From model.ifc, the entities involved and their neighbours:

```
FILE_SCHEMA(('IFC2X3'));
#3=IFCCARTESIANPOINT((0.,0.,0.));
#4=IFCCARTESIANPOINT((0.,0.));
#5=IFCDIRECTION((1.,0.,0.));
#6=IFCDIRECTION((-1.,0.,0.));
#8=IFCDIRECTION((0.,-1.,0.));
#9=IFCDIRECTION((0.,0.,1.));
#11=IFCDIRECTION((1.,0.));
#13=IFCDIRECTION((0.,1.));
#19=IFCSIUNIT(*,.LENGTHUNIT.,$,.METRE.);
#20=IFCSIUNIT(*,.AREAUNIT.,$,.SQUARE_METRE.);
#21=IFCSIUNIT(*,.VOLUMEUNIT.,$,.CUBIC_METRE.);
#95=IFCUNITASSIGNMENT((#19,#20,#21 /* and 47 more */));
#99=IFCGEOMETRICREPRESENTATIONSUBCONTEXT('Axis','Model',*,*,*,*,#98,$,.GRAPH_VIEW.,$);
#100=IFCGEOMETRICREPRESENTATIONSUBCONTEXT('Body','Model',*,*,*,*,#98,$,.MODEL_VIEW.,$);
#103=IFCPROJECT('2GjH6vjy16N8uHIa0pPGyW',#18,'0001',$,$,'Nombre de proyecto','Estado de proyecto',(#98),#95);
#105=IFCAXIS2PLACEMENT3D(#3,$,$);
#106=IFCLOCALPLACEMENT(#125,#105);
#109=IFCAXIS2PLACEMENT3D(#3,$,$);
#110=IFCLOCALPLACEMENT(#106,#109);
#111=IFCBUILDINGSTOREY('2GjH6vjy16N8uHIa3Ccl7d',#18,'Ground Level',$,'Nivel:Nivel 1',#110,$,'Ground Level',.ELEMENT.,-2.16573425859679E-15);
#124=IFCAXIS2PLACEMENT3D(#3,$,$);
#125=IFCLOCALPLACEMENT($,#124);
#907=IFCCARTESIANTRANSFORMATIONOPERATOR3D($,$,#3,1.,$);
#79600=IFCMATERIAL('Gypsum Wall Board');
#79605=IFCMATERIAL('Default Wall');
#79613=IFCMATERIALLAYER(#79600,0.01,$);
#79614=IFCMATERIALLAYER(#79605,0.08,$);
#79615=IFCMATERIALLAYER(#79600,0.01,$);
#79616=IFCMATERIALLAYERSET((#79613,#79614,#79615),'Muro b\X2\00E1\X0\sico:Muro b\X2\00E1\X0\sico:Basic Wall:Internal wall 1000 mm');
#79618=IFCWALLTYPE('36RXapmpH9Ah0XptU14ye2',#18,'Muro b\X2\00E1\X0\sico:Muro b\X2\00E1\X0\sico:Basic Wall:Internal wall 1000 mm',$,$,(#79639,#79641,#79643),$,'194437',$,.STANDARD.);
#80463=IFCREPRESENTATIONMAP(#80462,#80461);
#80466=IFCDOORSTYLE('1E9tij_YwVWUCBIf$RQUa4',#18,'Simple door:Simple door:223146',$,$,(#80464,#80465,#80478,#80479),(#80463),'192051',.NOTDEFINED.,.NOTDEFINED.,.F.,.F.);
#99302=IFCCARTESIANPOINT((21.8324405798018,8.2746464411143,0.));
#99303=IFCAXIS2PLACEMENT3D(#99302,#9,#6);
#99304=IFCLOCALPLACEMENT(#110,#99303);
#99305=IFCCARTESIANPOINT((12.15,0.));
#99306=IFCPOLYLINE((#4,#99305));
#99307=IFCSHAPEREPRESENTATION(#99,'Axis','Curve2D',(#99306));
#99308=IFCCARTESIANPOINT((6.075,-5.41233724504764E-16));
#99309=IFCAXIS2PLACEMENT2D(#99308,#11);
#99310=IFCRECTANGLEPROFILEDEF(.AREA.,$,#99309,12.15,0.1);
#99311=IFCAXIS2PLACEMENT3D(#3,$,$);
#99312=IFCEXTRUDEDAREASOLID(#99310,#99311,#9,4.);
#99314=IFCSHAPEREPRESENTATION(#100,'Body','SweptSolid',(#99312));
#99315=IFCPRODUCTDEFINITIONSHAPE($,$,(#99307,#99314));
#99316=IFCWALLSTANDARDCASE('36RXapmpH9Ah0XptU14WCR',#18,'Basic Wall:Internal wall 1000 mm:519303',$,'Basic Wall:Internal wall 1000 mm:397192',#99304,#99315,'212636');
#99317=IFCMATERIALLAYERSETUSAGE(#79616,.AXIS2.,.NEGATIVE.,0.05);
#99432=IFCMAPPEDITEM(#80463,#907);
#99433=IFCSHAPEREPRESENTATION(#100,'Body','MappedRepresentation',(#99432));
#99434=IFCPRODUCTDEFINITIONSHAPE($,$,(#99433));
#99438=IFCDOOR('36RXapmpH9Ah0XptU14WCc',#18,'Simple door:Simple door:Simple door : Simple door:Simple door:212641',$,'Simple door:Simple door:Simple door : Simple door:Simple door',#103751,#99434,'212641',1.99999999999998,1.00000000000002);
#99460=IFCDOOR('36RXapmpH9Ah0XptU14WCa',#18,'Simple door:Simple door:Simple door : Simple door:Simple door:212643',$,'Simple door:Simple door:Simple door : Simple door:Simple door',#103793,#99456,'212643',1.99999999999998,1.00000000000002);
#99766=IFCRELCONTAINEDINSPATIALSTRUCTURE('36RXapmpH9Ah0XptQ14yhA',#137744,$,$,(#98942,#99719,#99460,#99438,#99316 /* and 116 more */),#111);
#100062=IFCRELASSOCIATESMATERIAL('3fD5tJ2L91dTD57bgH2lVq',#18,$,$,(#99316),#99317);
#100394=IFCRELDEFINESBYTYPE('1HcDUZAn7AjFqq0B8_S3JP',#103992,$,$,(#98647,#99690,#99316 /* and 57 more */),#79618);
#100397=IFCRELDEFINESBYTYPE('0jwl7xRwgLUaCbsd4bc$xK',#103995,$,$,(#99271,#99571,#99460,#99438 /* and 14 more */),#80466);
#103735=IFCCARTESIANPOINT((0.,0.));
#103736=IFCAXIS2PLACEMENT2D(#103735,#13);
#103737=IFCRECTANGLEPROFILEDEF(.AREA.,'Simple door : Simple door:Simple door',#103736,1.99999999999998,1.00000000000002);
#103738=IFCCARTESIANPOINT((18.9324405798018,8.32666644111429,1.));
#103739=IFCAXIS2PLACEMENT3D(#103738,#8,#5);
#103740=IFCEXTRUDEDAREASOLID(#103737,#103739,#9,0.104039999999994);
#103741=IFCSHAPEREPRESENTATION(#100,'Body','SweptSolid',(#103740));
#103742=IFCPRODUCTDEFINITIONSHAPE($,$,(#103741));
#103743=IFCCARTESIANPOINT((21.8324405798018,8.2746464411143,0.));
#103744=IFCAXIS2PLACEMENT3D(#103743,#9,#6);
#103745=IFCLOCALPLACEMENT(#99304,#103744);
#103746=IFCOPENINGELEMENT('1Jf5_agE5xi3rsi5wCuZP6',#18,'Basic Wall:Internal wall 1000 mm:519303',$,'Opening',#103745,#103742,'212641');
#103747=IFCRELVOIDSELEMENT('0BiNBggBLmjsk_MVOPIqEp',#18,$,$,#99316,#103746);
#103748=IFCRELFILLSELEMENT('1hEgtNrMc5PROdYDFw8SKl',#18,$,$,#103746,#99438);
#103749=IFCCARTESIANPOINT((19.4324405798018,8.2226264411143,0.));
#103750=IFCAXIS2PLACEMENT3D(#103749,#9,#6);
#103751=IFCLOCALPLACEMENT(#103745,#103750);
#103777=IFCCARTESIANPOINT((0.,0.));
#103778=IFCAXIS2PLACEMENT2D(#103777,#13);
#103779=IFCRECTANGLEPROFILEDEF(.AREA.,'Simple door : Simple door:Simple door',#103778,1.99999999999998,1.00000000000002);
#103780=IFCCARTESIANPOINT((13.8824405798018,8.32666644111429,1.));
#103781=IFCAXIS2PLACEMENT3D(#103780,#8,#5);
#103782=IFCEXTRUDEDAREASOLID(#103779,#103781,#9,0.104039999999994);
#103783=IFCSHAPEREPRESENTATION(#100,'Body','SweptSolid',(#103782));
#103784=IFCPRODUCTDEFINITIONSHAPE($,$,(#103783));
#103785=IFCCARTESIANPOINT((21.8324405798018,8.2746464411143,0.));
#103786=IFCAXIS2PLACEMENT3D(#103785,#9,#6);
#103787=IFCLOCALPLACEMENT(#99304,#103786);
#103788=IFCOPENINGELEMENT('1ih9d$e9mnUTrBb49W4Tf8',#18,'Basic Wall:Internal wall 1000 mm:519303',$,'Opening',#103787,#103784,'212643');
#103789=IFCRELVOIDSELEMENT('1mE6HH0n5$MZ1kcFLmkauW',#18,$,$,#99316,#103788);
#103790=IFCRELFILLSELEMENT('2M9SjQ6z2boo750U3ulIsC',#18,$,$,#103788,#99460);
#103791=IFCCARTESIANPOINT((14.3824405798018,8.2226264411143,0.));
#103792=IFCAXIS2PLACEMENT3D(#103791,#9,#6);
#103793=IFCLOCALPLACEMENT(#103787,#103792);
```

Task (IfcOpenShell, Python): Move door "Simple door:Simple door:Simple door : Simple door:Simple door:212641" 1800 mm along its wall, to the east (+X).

```python
import ifcopenshell
import ifcopenshell.api.geometry
import ifcopenshell.util.placement

model = ifcopenshell.open("model.ifc")

door = model.by_guid("36RXapmpH9Ah0XptU14WCc")
opening = door.FillsVoids[0].RelatingOpeningElement
wall = opening.VoidsElements[0].RelatingBuildingElement

wall_matrix = ifcopenshell.util.placement.get_local_placement(wall.ObjectPlacement)
shift = wall_matrix[:3, 0] * -1.8
before = ifcopenshell.util.placement.get_local_placement(door.ObjectPlacement)[:3, 3].copy()

# The door is placed relative to its opening, so it follows when the opening moves.
matrix = ifcopenshell.util.placement.get_local_placement(opening.ObjectPlacement)
matrix[:3, 3] += shift
ifcopenshell.api.geometry.edit_object_placement(
    model, product=opening, matrix=matrix, is_si=False, should_transform_children=True
)

after = ifcopenshell.util.placement.get_local_placement(door.ObjectPlacement)[:3, 3]
print("door moved by", (after - before).round(3) + 0.0)

model.write("model-out.ifc")
```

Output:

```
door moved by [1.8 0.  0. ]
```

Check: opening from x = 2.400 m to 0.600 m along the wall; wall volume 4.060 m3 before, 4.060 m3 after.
